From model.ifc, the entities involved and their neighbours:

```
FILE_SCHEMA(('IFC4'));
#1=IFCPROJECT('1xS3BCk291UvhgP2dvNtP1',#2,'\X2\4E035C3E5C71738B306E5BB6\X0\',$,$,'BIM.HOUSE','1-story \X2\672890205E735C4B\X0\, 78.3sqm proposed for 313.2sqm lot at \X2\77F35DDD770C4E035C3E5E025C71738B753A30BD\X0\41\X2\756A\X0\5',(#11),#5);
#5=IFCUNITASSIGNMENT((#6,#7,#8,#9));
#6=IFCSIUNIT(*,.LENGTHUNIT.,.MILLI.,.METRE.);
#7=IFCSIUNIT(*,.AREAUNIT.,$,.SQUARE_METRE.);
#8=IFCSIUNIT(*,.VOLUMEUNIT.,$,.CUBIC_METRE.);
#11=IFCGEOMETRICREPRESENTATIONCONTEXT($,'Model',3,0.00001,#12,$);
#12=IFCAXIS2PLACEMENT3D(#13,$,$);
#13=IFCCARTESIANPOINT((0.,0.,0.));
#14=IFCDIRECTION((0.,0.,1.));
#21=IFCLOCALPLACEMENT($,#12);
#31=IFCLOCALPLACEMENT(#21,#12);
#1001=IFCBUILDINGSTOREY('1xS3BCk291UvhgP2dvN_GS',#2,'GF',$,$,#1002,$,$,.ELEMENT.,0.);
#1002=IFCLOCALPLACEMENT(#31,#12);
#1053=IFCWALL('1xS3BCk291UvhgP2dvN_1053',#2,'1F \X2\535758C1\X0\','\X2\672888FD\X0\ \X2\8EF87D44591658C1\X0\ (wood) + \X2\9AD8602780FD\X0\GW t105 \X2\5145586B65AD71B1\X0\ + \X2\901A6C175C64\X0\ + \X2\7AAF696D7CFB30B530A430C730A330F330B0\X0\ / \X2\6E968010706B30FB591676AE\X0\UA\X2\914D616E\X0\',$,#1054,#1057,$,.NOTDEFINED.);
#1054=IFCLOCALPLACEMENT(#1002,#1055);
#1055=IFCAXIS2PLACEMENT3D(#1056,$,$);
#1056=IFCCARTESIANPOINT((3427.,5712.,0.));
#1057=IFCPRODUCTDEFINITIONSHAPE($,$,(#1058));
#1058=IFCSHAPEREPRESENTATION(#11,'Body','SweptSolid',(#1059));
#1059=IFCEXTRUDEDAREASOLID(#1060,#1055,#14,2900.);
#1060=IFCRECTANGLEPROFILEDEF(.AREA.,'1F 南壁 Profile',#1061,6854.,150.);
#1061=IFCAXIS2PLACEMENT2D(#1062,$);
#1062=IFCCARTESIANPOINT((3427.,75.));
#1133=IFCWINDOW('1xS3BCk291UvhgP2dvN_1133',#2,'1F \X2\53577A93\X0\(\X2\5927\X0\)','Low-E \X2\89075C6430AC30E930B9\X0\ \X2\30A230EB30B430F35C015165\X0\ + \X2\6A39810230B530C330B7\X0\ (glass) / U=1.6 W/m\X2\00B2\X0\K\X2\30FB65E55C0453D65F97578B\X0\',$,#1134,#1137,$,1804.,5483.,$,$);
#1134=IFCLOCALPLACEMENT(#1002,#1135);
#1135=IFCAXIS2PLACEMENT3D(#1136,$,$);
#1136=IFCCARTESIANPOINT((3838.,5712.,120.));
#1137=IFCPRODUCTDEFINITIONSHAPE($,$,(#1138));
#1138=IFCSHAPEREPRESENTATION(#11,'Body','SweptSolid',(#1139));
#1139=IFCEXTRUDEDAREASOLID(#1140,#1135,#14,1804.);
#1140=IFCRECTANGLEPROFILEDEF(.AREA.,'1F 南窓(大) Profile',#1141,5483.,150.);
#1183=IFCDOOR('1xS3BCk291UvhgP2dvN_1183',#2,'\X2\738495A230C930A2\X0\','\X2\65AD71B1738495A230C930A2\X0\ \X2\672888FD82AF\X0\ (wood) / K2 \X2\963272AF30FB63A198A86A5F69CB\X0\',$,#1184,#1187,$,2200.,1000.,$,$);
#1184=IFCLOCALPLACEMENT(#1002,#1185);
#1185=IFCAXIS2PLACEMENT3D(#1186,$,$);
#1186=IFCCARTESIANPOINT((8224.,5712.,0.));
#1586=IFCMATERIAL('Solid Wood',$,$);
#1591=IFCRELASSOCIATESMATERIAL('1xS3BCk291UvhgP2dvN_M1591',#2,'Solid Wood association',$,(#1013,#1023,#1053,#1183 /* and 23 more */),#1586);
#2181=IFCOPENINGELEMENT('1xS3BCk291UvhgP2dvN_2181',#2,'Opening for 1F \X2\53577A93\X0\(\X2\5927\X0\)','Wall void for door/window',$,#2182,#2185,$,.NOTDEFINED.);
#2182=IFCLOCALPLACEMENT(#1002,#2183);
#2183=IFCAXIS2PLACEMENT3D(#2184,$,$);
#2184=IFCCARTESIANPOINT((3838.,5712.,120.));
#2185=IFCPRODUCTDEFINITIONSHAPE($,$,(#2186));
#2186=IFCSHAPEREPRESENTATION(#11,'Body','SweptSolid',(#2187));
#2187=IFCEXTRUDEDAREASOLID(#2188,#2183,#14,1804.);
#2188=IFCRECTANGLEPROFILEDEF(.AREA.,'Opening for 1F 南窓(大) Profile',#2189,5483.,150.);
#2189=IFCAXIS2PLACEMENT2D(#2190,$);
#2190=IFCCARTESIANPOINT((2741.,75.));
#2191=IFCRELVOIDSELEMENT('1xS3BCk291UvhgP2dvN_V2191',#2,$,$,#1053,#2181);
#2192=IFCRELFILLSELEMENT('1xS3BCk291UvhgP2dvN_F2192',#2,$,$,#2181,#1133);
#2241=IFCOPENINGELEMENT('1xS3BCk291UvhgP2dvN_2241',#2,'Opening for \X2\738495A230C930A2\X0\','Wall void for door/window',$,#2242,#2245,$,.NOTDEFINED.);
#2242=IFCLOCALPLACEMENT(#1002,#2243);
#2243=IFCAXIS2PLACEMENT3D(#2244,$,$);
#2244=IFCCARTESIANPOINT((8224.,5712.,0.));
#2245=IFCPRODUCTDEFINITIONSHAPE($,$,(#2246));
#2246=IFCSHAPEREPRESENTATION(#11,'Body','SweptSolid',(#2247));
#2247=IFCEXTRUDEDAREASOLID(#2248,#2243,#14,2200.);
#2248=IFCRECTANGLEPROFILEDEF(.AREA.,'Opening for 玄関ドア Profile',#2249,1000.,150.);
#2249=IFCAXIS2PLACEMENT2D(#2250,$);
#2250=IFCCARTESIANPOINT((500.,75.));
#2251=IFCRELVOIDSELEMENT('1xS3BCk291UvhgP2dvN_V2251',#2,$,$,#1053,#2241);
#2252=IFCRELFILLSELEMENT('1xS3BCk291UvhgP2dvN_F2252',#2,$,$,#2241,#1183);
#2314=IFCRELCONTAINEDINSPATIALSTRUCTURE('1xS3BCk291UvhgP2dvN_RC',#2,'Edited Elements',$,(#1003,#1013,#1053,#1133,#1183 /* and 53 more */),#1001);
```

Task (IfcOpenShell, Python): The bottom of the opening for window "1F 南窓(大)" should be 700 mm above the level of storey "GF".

```python
import numpy as np
import ifcopenshell
import ifcopenshell.api.geometry
import ifcopenshell.geom
import ifcopenshell.util.element
import ifcopenshell.util.placement
import ifcopenshell.util.shape
import ifcopenshell.util.unit

model = ifcopenshell.open("model.ifc")
unit_scale = ifcopenshell.util.unit.calculate_unit_scale(model)

window = model.by_guid("1xS3BCk291UvhgP2dvN_1133")
opening = window.FillsVoids[0].RelatingOpeningElement
storey = ifcopenshell.util.element.get_container(window, ifc_class="IfcBuildingStorey")
level = ifcopenshell.util.placement.get_local_placement(storey.ObjectPlacement)[2, 3]

# The opening's origin need not be at the sill, so measure its lowest point.
shape = ifcopenshell.geom.create_shape(ifcopenshell.geom.settings(), opening)
bottom = ifcopenshell.util.shape.get_shape_bottom_elevation(shape, shape.geometry) / unit_scale
dz = level + 0.7 / unit_scale - bottom

shift = np.array([0.0, 0.0, dz])
# The window is not placed relative to its opening, so move both.
for product in (opening, window):
    matrix = ifcopenshell.util.placement.get_local_placement(product.ObjectPlacement)
    matrix[:3, 3] += shift
    ifcopenshell.api.geometry.edit_object_placement(model, product=product, matrix=matrix, is_si=False)

print(f"moved by {dz * unit_scale:+.3f} m")

model.write("model-out.ifc")
```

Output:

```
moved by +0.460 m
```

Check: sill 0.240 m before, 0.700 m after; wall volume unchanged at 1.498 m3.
